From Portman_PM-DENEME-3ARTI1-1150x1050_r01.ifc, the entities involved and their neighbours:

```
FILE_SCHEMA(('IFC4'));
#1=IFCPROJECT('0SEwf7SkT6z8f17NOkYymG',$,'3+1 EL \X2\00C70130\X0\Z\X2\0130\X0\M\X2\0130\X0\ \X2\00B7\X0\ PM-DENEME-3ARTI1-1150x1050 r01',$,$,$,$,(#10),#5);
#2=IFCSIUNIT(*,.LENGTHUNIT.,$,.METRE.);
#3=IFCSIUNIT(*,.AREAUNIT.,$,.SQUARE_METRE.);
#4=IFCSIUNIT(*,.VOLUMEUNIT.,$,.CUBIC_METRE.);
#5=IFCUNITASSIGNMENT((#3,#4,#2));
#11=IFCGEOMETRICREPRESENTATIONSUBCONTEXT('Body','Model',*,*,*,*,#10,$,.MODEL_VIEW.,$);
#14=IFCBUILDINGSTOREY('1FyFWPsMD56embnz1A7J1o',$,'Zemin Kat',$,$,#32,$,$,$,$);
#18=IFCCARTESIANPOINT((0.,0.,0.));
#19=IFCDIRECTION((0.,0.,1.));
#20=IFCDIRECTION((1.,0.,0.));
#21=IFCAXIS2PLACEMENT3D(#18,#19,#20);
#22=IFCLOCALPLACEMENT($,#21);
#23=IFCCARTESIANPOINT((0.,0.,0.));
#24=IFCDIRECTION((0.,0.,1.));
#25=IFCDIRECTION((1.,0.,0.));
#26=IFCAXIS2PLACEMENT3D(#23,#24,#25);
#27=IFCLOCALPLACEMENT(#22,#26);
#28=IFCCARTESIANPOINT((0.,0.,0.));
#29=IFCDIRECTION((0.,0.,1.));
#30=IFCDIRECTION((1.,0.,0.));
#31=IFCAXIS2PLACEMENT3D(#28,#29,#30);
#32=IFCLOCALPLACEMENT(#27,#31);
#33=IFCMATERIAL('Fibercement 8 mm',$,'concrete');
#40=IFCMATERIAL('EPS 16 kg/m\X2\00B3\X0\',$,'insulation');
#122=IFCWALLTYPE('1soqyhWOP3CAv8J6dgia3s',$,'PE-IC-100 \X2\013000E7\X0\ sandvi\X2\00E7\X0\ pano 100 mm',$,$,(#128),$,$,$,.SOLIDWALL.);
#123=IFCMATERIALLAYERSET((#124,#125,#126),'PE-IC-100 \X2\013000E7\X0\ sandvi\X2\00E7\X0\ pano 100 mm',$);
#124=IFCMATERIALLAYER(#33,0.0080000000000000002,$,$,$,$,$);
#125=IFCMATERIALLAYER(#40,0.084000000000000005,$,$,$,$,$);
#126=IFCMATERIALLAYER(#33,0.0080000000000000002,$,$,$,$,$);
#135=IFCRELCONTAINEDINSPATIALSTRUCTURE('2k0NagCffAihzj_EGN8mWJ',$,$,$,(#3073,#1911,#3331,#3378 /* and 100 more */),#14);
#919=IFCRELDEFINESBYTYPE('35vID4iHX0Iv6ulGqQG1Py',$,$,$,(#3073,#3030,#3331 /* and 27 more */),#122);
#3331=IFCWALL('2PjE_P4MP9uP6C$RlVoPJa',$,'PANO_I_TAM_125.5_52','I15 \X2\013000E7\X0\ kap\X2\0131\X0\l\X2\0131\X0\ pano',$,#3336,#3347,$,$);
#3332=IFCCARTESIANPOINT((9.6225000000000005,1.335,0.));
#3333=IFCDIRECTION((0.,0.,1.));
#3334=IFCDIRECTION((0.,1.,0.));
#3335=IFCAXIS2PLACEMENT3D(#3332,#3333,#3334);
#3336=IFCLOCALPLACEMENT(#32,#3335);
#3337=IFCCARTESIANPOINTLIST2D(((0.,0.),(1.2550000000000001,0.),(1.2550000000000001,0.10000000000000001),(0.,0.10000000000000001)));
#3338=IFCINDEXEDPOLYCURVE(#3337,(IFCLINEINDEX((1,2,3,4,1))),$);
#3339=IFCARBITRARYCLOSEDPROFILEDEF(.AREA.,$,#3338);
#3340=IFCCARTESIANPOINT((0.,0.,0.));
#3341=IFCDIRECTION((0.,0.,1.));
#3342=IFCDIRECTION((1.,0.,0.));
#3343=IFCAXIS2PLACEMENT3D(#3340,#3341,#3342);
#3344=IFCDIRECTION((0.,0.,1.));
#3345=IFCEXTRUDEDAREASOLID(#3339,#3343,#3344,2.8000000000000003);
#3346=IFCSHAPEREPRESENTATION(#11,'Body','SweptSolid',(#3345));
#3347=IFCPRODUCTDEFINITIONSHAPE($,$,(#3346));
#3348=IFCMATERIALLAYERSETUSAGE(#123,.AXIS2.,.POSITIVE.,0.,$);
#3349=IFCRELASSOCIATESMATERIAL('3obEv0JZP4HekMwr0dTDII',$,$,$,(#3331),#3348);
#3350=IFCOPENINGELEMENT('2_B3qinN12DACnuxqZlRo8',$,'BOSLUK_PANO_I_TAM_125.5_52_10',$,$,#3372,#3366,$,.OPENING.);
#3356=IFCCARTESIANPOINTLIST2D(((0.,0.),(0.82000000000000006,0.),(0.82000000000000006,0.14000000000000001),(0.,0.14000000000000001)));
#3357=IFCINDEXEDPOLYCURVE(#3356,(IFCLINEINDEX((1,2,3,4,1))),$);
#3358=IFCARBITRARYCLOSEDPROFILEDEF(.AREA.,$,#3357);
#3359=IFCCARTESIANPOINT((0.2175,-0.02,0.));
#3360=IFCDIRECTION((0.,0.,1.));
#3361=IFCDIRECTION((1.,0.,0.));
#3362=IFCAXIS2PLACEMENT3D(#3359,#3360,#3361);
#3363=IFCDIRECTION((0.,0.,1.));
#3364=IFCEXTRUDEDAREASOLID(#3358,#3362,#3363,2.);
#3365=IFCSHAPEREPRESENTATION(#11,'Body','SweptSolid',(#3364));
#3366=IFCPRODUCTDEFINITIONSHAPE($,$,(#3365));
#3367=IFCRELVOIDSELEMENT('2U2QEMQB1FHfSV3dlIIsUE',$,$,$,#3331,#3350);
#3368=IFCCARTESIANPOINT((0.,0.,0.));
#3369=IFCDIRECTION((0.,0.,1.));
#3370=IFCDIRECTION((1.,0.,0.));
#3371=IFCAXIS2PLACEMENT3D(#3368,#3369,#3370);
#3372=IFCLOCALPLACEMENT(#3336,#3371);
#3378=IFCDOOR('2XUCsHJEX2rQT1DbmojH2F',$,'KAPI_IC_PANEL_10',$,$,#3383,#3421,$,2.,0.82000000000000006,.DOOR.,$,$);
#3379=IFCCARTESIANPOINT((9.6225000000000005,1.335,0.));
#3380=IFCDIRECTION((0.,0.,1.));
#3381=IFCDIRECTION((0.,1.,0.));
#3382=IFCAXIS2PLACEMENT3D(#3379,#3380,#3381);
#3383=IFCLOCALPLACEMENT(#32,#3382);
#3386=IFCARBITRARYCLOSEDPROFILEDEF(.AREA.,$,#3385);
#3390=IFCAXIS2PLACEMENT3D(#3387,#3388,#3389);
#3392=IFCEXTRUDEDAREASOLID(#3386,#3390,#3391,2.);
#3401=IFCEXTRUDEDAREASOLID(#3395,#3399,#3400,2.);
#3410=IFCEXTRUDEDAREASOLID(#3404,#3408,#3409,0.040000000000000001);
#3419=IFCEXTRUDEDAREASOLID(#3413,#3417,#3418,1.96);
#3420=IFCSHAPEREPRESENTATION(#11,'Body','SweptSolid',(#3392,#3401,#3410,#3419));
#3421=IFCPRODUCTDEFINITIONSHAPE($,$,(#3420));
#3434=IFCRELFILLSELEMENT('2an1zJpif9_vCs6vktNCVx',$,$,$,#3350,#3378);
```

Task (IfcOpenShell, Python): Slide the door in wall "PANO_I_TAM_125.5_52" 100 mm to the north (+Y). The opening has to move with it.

```python
import ifcopenshell
import ifcopenshell.api.geometry
import ifcopenshell.util.placement
import ifcopenshell.util.unit

model = ifcopenshell.open("Portman_PM-DENEME-3ARTI1-1150x1050_r01.ifc")
unit_scale = ifcopenshell.util.unit.calculate_unit_scale(model)

door = model.by_guid("2XUCsHJEX2rQT1DbmojH2F")
opening = door.FillsVoids[0].RelatingOpeningElement
wall = opening.VoidsElements[0].RelatingBuildingElement

wall_matrix = ifcopenshell.util.placement.get_local_placement(wall.ObjectPlacement)
shift = wall_matrix[:3, 0] * 0.1 / unit_scale
before = ifcopenshell.util.placement.get_local_placement(door.ObjectPlacement)[:3, 3].copy()

# The door is not placed relative to its opening, so move both.
for product in (opening, door):
    matrix = ifcopenshell.util.placement.get_local_placement(product.ObjectPlacement)
    matrix[:3, 3] += shift
    ifcopenshell.api.geometry.edit_object_placement(model, product=product, matrix=matrix, is_si=False)

after = ifcopenshell.util.placement.get_local_placement(door.ObjectPlacement)[:3, 3]
print("door moved by", (after - before).round(3) + 0.0)

model.write("Portman_PM-DENEME-3ARTI1-1150x1050_r01_updated.ifc")
```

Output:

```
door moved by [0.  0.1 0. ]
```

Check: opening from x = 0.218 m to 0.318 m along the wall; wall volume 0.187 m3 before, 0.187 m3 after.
